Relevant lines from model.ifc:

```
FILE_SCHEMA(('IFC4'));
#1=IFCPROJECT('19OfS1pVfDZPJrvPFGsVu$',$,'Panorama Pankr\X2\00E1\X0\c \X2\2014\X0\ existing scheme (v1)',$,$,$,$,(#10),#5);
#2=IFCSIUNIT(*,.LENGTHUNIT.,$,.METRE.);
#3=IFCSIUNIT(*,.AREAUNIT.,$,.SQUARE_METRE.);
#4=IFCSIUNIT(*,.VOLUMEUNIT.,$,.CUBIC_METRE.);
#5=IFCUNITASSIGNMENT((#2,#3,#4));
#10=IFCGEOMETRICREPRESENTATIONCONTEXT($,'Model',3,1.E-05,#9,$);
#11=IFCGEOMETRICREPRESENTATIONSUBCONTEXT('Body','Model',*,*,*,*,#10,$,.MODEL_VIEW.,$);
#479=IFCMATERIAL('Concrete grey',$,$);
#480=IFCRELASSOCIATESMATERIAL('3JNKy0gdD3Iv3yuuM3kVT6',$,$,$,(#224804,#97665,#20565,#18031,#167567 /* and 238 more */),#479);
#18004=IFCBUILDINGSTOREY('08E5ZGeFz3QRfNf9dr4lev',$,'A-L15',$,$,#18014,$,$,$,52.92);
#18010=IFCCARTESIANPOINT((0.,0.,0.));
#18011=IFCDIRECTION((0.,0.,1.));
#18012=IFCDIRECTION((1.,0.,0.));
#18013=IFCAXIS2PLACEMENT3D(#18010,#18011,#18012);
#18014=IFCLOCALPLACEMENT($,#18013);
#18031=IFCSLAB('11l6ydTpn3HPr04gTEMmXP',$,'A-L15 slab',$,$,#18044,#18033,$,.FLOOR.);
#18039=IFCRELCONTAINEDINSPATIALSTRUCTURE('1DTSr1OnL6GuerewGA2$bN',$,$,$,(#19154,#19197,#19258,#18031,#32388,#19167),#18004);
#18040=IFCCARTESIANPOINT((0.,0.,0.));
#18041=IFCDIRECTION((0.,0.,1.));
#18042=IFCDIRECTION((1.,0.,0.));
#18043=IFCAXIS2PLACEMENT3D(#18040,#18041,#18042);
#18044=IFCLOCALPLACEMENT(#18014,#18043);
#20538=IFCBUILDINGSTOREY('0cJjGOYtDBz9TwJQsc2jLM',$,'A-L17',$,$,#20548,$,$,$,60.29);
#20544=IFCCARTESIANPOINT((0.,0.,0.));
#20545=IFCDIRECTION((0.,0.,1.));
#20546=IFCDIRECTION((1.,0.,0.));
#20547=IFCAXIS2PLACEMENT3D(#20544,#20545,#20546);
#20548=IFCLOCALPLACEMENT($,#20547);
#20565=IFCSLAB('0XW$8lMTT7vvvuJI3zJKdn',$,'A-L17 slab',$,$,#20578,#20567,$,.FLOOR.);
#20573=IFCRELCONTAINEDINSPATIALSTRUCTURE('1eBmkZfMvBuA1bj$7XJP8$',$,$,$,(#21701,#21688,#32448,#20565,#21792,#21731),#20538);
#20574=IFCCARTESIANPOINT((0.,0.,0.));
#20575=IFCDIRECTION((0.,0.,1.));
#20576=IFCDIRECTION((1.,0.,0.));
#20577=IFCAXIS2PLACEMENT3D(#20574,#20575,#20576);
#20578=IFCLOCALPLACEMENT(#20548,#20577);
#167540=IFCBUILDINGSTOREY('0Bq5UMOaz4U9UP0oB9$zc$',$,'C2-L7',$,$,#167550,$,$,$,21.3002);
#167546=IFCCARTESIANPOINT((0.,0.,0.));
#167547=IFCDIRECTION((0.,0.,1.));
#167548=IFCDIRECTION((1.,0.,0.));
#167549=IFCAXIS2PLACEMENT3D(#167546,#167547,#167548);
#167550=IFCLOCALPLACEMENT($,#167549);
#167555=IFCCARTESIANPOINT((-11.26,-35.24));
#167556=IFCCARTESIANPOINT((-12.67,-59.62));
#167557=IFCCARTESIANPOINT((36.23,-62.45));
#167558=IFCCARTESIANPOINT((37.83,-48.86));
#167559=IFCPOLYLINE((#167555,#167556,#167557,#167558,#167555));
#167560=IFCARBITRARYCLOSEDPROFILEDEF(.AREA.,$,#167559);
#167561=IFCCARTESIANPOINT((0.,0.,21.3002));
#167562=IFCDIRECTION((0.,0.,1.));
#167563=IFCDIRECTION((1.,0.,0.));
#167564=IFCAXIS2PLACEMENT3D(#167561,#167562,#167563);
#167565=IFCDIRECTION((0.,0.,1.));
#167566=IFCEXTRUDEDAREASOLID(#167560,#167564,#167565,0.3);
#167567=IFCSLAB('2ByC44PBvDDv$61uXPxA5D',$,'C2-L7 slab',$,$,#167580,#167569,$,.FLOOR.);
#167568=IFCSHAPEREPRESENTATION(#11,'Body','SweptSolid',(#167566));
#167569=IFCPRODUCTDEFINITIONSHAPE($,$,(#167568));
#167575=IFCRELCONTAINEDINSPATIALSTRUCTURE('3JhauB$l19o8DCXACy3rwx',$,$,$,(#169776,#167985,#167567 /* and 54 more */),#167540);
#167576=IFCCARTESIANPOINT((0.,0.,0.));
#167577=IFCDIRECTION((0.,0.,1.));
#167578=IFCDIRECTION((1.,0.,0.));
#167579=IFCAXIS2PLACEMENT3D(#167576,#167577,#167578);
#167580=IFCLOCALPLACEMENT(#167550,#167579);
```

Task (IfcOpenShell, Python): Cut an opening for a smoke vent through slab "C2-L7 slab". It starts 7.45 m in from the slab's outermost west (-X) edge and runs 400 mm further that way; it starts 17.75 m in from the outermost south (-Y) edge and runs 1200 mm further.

```python
import numpy as np
import ifcopenshell
import ifcopenshell.api.feature
import ifcopenshell.api.geometry
import ifcopenshell.api.root
import ifcopenshell.geom
import ifcopenshell.util.placement
import ifcopenshell.util.representation
import ifcopenshell.util.shape
import ifcopenshell.util.unit

model = ifcopenshell.open("model.ifc")
unit_scale = ifcopenshell.util.unit.calculate_unit_scale(model)
settings = ifcopenshell.geom.settings()


def volume(element):
    """Net volume in cubic metres, openings subtracted."""
    shape = ifcopenshell.geom.create_shape(settings, element)
    return ifcopenshell.util.shape.get_volume(shape.geometry)


slab = model.by_guid("2ByC44PBvDDv$61uXPxA5D")
before = volume(slab)

# Extent in the slab's own axes, in metres. The edges named are its -X and -Y sides.
slab_shape = ifcopenshell.geom.create_shape(settings, slab)
vertices = ifcopenshell.util.shape.get_vertices(slab_shape.geometry)
x_min, y_min, bottom = vertices.min(axis=0)
top = vertices[:, 2].max()

opening = ifcopenshell.api.root.create_entity(model, ifc_class="IfcOpeningElement", name="Smoke vent opening", predefined_type="OPENING")
context = ifcopenshell.util.representation.get_context(model, "Model", "Body", "MODEL_VIEW")
width, depth = 0.4, 1.2
outline = [(0.0, 0.0), (width, 0.0), (width, depth), (0.0, depth), (0.0, 0.0)]
# Overshoot both faces by 50 mm so the cut is clean.
shape = ifcopenshell.api.geometry.add_slab_representation(
    model, context=context, depth=top - bottom + 0.1, polyline=outline
)
ifcopenshell.api.geometry.assign_representation(model, product=opening, representation=shape)

matrix = ifcopenshell.util.placement.get_local_placement(slab.ObjectPlacement)
matrix[:, 3] = matrix @ np.append(np.array([x_min + 7.45, y_min + 17.75, bottom - 0.05]) / unit_scale, 1.0)
ifcopenshell.api.geometry.edit_object_placement(model, product=opening, matrix=matrix, is_si=False)
ifcopenshell.api.feature.add_feature(model, feature=opening, element=slab)

after = volume(slab)

print(f"slab volume {before:.3f} -> {after:.3f} m3")

model.write("model_edited.ifc")
```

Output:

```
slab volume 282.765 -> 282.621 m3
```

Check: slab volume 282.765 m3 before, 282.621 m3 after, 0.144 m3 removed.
